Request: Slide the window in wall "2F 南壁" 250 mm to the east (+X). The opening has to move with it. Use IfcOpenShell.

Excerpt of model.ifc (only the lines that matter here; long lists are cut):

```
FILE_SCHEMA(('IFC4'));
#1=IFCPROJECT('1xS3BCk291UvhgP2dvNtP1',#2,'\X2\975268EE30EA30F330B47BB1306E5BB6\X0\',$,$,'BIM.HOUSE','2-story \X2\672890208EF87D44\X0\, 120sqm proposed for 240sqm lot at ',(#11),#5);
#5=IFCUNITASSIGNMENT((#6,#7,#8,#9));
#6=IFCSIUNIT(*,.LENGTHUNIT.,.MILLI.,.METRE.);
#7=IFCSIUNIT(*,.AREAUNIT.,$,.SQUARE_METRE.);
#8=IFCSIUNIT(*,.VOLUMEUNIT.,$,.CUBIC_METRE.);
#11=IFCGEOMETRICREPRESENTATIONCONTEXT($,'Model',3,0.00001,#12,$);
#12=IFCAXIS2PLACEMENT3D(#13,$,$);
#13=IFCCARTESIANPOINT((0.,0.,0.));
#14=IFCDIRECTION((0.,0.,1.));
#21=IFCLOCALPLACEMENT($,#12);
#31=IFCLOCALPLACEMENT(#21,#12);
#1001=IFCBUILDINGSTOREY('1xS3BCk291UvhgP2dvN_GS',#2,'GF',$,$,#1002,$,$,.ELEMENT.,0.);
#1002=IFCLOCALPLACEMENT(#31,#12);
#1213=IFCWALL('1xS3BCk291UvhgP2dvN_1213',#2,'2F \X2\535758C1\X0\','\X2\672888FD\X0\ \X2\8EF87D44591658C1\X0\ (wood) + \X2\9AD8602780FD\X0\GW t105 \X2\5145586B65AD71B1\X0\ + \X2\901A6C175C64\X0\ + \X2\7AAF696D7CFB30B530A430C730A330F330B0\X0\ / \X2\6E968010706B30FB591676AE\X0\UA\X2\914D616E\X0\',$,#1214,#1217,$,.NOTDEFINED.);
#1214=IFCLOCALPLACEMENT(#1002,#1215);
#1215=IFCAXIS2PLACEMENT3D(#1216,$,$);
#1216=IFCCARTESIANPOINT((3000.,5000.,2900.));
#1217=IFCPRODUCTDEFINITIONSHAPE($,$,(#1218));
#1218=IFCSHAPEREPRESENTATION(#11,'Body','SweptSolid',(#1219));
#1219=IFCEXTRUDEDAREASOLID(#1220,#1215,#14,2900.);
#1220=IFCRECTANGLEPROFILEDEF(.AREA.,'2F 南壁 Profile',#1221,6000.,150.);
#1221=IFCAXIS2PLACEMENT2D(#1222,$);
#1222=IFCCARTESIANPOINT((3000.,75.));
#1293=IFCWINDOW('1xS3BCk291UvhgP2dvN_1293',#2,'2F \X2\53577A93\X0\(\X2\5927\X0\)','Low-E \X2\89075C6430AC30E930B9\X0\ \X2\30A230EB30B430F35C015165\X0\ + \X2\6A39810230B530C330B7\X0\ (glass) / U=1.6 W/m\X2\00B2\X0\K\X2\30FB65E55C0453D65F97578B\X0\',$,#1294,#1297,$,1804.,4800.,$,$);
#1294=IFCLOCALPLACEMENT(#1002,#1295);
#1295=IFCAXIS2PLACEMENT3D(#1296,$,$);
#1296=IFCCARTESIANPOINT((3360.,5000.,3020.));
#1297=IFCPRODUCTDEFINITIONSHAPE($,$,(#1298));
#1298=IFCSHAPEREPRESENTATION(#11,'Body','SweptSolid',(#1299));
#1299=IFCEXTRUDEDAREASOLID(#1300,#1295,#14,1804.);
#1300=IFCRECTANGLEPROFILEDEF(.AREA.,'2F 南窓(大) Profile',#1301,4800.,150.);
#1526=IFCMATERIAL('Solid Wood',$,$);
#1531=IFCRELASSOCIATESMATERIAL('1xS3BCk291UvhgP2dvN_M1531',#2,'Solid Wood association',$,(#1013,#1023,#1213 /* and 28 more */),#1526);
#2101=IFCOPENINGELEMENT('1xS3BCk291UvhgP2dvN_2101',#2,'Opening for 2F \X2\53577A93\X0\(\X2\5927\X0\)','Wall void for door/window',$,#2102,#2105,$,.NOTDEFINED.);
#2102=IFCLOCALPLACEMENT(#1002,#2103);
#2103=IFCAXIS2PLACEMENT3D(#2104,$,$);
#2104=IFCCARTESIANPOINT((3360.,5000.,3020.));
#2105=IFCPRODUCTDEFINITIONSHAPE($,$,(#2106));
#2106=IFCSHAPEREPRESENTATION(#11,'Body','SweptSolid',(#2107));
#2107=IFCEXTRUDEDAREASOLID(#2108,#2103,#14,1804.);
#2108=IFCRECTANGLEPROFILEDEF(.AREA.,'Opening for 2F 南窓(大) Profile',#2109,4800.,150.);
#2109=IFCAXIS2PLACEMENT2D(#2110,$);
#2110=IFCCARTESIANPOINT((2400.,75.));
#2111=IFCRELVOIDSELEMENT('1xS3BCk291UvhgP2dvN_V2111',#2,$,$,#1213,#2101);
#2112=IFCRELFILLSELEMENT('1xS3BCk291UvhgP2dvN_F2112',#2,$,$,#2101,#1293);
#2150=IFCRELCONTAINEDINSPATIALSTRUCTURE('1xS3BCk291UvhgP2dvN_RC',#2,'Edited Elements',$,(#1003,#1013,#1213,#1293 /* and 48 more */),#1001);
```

```python
import ifcopenshell
import ifcopenshell.api.geometry
import ifcopenshell.util.placement
import ifcopenshell.util.unit

model = ifcopenshell.open("model.ifc")
unit_scale = ifcopenshell.util.unit.calculate_unit_scale(model)

window = model.by_guid("1xS3BCk291UvhgP2dvN_1293")
opening = window.FillsVoids[0].RelatingOpeningElement
wall = opening.VoidsElements[0].RelatingBuildingElement

wall_matrix = ifcopenshell.util.placement.get_local_placement(wall.ObjectPlacement)
shift = wall_matrix[:3, 0] * 0.25 / unit_scale
before = ifcopenshell.util.placement.get_local_placement(window.ObjectPlacement)[:3, 3].copy()

# The window is not placed relative to its opening, so move both.
for product in (opening, window):
    matrix = ifcopenshell.util.placement.get_local_placement(product.ObjectPlacement)
    matrix[:3, 3] += shift
    ifcopenshell.api.geometry.edit_object_placement(model, product=product, matrix=matrix, is_si=False)

after = ifcopenshell.util.placement.get_local_placement(window.ObjectPlacement)[:3, 3]
print("window moved by", (after - before).round(3) + 0.0)

model.write("model_rev.ifc")
```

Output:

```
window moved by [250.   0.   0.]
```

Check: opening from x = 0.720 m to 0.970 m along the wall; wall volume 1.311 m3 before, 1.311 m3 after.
